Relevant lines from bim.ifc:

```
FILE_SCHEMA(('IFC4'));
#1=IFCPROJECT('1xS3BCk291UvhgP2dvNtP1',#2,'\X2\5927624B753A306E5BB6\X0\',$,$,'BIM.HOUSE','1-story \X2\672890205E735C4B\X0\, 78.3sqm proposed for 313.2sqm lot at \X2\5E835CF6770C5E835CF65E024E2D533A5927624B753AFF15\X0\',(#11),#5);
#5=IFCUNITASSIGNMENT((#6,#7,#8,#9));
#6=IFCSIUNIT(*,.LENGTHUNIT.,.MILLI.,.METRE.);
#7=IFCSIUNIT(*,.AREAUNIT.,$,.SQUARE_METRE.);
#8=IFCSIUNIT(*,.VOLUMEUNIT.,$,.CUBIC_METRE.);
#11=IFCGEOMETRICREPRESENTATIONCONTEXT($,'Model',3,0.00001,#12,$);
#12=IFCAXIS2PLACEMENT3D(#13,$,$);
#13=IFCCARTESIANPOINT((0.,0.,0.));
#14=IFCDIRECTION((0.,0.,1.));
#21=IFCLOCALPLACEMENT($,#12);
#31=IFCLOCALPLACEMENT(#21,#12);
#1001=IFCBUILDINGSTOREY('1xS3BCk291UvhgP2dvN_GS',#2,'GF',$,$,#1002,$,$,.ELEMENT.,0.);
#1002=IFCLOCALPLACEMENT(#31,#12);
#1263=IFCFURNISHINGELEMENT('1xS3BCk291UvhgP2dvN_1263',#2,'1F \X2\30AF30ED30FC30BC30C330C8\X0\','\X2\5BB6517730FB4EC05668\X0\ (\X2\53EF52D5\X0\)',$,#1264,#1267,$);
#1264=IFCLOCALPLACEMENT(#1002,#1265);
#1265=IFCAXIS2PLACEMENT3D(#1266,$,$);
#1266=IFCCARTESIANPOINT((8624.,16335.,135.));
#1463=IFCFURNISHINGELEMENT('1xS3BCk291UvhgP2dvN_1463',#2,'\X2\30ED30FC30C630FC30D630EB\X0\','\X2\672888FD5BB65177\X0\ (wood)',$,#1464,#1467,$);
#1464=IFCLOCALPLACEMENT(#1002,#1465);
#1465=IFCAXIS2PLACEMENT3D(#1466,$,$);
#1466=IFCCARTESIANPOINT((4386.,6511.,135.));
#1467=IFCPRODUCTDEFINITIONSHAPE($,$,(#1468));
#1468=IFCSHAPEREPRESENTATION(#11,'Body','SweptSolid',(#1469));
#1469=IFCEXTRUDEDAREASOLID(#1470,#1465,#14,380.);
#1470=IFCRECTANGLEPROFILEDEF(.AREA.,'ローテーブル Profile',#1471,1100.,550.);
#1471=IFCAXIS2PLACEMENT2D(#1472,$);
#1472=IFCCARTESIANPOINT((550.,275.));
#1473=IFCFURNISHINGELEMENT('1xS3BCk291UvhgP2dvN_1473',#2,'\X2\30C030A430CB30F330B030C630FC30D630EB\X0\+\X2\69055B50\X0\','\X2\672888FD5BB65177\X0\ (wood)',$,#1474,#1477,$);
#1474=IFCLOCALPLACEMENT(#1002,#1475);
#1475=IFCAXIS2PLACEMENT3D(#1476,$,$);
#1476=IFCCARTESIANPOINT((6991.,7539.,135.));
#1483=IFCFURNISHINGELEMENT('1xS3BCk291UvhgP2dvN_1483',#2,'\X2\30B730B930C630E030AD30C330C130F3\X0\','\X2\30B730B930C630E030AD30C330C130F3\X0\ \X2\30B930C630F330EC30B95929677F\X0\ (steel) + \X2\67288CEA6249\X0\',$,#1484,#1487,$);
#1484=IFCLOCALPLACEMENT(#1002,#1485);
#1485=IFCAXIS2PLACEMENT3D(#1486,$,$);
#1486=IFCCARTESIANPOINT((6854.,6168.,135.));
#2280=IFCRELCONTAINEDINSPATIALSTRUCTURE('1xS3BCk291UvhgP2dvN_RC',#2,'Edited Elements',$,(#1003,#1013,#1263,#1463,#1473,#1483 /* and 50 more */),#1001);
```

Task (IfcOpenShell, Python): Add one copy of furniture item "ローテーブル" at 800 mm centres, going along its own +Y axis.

```python
import ifcopenshell
import ifcopenshell.api.geometry
import ifcopenshell.api.root
import ifcopenshell.util.element
import ifcopenshell.util.placement
import ifcopenshell.util.unit

model = ifcopenshell.open("bim.ifc")
unit_scale = ifcopenshell.util.unit.calculate_unit_scale(model)


def reuse_history(source, copy):
    """copy_class also copies each property set's owner history, people and application; keep the originals."""
    for rel in copy.IsDefinedBy:
        if rel.is_a("IfcRelDefinesByProperties") and (history := rel.RelatingPropertyDefinition.OwnerHistory):
            rel.RelatingPropertyDefinition.OwnerHistory = source.OwnerHistory
            ifcopenshell.util.element.remove_deep2(model, history)


source = model.by_guid("1xS3BCk291UvhgP2dvN_1463")
base = ifcopenshell.util.placement.get_local_placement(source.ObjectPlacement)
step = base[:3, 1] * 0.8 / unit_scale

for i in range(1, 2):
    copy = ifcopenshell.api.root.copy_class(model, product=source)
    copy.Representation = ifcopenshell.util.element.copy_deep(
        model, source.Representation, exclude=["IfcGeometricRepresentationContext", "IfcRepresentationMap"]
    )
    reuse_history(source, copy)
    matrix = base.copy()
    matrix[:3, 3] += i * step
    print("added at", matrix[:3, 3].round(3) + 0.0)
    ifcopenshell.api.geometry.edit_object_placement(model, product=copy, matrix=matrix, is_si=False)

model.write("bim-out.ifc")
```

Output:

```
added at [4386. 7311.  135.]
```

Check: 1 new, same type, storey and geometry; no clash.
